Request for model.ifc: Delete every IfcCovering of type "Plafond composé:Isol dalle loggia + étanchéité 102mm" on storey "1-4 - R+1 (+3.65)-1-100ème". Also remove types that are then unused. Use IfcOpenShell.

First a look at what the model holds.

```python
import ifcopenshell
import ifcopenshell.util.element

model = ifcopenshell.open("model.ifc")
print(model.schema)
storey = next(s for s in model.by_type("IfcBuildingStorey") if s.Name == "1-4 - R+1 (+3.65)-1-100ème")
coverings = [e for e in ifcopenshell.util.element.get_decomposition(storey) if e.is_a("IfcCovering")]
seen = {}
for e in coverings:
    element_type = ifcopenshell.util.element.get_type(e)
    name = element_type.Name if element_type not in (None, e) else None
    seen[name] = seen.get(name, 0) + 1
for name, count in sorted(seen.items(), key=str):
    print(count, "x", name)
```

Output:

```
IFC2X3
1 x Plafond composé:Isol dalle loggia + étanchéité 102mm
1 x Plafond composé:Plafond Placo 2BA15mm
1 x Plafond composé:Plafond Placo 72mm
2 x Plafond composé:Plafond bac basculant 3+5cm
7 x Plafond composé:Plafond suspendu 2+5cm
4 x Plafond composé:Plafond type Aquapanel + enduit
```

```python
import ifcopenshell
import ifcopenshell.api.root
import ifcopenshell.util.element

model = ifcopenshell.open("model.ifc")

storey = next(s for s in model.by_type("IfcBuildingStorey") if s.Name == "1-4 - R+1 (+3.65)-1-100ème")
coverings = [e for e in ifcopenshell.util.element.get_decomposition(storey) if e.is_a("IfcCovering")]
targets = [e for e in coverings if (t := ifcopenshell.util.element.get_type(e)) not in (None, e) and t.Name == "Plafond composé:Isol dalle loggia + étanchéité 102mm"]
types = {ifcopenshell.util.element.get_type(e) for e in targets} - {None, *targets}

for e in targets:
    ifcopenshell.api.root.remove_product(model, product=e)
print(len(targets), "removed")

unused = [t for t in types if not ifcopenshell.util.element.get_types(t)]
for t in unused:
    ifcopenshell.api.root.remove_product(model, product=t)
print(len(unused), "unused types removed")

model.write("model_v2.ifc")
```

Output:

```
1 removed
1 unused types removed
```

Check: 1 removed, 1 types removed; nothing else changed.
